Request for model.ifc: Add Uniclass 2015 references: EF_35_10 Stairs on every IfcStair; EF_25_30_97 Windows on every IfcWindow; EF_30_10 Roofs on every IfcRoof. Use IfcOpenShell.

First a look at what the model holds.

```python
import ifcopenshell

model = ifcopenshell.open("model.ifc")
print(model.schema)
print("classifications:", [c.Name for c in model.by_type("IfcClassification")])
for ifc_class in ("IfcDoor", "IfcRoof", "IfcStair", "IfcWall", "IfcWindow"):
    print(ifc_class, len(model.by_type(ifc_class)))
```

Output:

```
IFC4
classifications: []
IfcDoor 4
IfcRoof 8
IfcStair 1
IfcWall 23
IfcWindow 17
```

```python
import ifcopenshell
import ifcopenshell.api.classification

model = ifcopenshell.open("model.ifc")

system = ifcopenshell.api.classification.add_classification(model, classification="Uniclass 2015")

codes = {
    "IfcStair": ("EF_35_10", "Stairs"),
    "IfcWindow": ("EF_25_30_97", "Windows"),
    "IfcRoof": ("EF_30_10", "Roofs"),
}
for ifc_class, (code, name) in codes.items():
    products = model.by_type(ifc_class)
    ifcopenshell.api.classification.add_reference(
        model, products=products, classification=system, identification=code, name=name
    )
    print(code, len(products))

model.write("model_updated.ifc")
```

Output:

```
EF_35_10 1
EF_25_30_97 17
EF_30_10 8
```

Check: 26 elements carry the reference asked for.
